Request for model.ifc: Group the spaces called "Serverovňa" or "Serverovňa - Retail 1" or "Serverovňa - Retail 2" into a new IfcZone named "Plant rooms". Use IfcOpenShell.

First a look at what the model holds.

```python
import ifcopenshell

model = ifcopenshell.open("model.ifc")
print(model.schema)
seen = {}
for space in model.by_type("IfcSpace"):
    seen[space.LongName] = seen.get(space.LongName, 0) + 1
for name, count in sorted(seen.items(), key=str):
    print(count, "x", name)
print("zones:", [z.Name for z in model.by_type("IfcZone")][:20])
```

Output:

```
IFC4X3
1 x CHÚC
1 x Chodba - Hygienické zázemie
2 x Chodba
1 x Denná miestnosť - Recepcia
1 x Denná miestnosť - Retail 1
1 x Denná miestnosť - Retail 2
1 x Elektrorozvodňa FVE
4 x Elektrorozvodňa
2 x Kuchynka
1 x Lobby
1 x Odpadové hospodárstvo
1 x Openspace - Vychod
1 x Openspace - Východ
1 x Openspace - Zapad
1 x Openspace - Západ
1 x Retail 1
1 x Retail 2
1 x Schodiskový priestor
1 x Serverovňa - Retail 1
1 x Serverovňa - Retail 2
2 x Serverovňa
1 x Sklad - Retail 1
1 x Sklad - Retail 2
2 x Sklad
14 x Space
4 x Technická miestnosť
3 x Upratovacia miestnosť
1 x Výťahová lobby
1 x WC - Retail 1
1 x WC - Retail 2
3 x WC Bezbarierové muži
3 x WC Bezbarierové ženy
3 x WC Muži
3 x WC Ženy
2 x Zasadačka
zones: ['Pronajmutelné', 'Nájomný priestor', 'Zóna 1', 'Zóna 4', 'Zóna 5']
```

```python
import ifcopenshell
import ifcopenshell.api.group
import ifcopenshell.api.root

model = ifcopenshell.open("model.ifc")

names = {"Serverovňa", "Serverovňa - Retail 1", "Serverovňa - Retail 2"}
spaces = [s for s in model.by_type("IfcSpace") if s.LongName in names]

zone = ifcopenshell.api.root.create_entity(model, ifc_class="IfcZone", name="Plant rooms")
ifcopenshell.api.group.assign_group(model, products=spaces, group=zone)
print(len(spaces), "spaces in", zone.Name)

model.write("model_v2.ifc")
```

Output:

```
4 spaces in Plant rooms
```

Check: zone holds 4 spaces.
